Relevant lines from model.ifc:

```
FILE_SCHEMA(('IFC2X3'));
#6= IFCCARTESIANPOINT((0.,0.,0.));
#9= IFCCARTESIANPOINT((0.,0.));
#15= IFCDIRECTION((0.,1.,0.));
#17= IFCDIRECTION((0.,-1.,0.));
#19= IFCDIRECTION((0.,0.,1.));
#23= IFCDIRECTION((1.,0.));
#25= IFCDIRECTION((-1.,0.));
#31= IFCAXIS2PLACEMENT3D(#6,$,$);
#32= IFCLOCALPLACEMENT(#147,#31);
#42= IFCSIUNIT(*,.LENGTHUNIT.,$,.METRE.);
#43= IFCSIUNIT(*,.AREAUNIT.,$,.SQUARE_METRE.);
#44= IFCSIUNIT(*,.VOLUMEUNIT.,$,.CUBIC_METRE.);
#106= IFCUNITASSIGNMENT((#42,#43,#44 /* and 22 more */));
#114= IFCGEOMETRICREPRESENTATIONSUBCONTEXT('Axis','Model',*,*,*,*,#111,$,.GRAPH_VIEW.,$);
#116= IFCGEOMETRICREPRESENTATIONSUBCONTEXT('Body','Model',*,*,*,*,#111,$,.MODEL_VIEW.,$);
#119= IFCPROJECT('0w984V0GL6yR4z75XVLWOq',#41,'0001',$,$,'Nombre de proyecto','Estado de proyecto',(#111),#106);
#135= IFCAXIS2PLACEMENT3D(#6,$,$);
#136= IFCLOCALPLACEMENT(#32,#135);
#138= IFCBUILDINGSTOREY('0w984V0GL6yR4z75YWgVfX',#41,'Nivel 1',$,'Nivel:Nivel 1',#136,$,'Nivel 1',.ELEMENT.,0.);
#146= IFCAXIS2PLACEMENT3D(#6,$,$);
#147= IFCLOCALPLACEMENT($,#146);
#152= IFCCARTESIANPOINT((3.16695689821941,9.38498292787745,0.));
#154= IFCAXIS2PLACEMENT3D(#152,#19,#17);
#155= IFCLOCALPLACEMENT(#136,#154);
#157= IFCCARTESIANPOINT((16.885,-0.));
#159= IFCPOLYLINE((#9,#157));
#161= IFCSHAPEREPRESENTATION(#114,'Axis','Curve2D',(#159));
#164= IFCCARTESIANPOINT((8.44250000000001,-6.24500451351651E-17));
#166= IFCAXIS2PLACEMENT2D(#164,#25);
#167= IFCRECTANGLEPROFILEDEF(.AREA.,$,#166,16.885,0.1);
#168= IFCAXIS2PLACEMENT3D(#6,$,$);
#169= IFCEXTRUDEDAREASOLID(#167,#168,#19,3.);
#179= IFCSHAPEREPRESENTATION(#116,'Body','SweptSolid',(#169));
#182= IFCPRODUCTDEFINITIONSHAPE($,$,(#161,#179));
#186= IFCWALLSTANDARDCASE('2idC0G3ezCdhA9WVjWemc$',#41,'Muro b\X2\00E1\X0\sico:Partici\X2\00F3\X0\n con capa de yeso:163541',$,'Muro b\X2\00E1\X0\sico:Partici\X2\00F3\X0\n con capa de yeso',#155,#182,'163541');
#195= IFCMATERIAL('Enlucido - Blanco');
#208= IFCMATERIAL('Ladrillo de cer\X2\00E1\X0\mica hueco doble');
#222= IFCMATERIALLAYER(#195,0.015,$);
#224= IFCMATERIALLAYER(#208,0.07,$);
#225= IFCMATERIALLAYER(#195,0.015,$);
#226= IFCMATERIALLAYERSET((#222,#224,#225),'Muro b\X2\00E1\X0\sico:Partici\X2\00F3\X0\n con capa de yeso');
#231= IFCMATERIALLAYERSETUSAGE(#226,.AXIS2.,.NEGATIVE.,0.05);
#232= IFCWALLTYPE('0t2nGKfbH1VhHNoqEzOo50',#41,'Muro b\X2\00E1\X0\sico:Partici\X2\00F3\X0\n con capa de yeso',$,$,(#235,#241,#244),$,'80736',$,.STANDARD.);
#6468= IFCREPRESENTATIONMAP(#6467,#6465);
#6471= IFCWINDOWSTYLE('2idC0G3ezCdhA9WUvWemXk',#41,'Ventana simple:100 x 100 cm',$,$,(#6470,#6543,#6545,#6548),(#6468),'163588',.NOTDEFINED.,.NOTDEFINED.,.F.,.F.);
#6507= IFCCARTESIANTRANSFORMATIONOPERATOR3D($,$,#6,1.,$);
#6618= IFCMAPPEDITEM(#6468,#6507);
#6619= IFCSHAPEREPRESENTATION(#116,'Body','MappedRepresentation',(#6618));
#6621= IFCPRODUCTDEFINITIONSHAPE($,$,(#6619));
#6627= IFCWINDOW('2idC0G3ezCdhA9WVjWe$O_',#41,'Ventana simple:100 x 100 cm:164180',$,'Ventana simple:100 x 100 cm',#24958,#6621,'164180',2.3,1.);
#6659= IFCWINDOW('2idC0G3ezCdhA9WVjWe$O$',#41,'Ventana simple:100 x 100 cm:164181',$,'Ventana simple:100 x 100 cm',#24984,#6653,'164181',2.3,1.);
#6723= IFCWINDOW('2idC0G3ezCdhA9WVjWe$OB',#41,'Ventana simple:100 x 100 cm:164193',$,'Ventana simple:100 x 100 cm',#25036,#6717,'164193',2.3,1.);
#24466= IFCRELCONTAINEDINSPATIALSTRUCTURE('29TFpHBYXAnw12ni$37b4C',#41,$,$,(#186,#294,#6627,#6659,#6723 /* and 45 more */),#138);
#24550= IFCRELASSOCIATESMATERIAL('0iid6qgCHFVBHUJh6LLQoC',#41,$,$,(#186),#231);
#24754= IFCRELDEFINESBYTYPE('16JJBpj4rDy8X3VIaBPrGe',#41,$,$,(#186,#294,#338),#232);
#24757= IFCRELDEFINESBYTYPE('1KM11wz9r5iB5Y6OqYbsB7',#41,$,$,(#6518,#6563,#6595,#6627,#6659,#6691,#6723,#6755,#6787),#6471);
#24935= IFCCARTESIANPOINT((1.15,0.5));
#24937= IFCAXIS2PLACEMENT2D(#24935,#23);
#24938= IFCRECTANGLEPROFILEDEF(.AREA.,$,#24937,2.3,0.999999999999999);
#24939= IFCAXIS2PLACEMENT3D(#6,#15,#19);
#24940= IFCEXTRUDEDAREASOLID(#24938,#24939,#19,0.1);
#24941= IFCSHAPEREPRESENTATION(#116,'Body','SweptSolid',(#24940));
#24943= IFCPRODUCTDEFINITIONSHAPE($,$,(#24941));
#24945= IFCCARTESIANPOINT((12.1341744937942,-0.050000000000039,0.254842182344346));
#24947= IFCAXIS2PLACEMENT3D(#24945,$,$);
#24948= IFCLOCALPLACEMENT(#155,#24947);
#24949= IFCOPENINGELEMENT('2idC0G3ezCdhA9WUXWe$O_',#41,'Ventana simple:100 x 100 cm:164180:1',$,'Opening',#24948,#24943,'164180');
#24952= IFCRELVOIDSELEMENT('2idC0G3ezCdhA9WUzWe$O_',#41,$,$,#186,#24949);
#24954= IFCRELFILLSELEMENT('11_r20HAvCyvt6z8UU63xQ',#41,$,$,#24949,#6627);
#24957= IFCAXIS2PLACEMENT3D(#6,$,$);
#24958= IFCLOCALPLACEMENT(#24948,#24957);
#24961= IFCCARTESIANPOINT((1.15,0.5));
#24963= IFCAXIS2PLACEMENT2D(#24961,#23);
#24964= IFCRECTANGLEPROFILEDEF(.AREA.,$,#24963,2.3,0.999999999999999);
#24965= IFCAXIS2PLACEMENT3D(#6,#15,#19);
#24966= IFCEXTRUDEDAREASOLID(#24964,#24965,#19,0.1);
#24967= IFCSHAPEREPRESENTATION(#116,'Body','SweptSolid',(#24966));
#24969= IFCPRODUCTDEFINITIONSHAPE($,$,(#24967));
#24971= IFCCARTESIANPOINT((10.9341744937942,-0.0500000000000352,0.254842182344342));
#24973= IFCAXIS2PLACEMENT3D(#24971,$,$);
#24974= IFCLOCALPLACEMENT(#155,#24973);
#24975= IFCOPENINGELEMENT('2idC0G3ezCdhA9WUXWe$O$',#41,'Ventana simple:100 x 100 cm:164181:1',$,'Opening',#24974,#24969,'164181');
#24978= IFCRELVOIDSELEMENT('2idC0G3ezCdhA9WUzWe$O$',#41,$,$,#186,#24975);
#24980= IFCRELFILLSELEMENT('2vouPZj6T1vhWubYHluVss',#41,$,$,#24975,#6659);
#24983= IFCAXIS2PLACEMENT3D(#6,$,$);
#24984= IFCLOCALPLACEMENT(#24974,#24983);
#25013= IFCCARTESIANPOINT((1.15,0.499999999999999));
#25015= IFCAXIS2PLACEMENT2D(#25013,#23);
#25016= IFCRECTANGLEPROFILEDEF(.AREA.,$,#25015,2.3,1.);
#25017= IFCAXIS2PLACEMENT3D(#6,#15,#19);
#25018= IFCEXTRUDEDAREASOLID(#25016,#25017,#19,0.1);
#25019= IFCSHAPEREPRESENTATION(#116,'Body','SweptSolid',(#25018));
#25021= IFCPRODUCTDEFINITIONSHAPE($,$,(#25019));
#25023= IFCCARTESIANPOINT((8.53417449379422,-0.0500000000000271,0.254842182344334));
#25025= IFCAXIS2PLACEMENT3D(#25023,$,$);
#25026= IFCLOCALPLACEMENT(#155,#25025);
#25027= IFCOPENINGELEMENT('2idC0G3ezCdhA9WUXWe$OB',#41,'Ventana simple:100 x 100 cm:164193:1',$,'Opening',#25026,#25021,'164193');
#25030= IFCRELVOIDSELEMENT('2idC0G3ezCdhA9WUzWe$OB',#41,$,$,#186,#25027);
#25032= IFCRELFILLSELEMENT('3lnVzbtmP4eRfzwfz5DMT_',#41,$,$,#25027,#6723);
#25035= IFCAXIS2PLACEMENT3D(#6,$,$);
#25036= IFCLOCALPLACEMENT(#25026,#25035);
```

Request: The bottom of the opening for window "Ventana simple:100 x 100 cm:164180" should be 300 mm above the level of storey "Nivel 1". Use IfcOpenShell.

```python
import numpy as np
import ifcopenshell
import ifcopenshell.api.geometry
import ifcopenshell.geom
import ifcopenshell.util.element
import ifcopenshell.util.placement
import ifcopenshell.util.shape
import ifcopenshell.util.unit

model = ifcopenshell.open("model.ifc")
unit_scale = ifcopenshell.util.unit.calculate_unit_scale(model)

window = model.by_guid("2idC0G3ezCdhA9WVjWe$O_")
opening = window.FillsVoids[0].RelatingOpeningElement
storey = ifcopenshell.util.element.get_container(window, ifc_class="IfcBuildingStorey")
level = ifcopenshell.util.placement.get_local_placement(storey.ObjectPlacement)[2, 3]

# The opening's origin need not be at the sill, so measure its lowest point.
shape = ifcopenshell.geom.create_shape(ifcopenshell.geom.settings(), opening)
bottom = ifcopenshell.util.shape.get_shape_bottom_elevation(shape, shape.geometry) / unit_scale
dz = level + 0.3 / unit_scale - bottom

shift = np.array([0.0, 0.0, dz])
# The window is placed relative to its opening, so it follows when the opening moves.
matrix = ifcopenshell.util.placement.get_local_placement(opening.ObjectPlacement)
matrix[:3, 3] += shift
ifcopenshell.api.geometry.edit_object_placement(
    model, product=opening, matrix=matrix, is_si=False, should_transform_children=True
)

print(f"moved by {dz * unit_scale:+.3f} m")

model.write("model_updated.ifc")
```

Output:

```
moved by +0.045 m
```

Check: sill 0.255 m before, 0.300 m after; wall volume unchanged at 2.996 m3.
